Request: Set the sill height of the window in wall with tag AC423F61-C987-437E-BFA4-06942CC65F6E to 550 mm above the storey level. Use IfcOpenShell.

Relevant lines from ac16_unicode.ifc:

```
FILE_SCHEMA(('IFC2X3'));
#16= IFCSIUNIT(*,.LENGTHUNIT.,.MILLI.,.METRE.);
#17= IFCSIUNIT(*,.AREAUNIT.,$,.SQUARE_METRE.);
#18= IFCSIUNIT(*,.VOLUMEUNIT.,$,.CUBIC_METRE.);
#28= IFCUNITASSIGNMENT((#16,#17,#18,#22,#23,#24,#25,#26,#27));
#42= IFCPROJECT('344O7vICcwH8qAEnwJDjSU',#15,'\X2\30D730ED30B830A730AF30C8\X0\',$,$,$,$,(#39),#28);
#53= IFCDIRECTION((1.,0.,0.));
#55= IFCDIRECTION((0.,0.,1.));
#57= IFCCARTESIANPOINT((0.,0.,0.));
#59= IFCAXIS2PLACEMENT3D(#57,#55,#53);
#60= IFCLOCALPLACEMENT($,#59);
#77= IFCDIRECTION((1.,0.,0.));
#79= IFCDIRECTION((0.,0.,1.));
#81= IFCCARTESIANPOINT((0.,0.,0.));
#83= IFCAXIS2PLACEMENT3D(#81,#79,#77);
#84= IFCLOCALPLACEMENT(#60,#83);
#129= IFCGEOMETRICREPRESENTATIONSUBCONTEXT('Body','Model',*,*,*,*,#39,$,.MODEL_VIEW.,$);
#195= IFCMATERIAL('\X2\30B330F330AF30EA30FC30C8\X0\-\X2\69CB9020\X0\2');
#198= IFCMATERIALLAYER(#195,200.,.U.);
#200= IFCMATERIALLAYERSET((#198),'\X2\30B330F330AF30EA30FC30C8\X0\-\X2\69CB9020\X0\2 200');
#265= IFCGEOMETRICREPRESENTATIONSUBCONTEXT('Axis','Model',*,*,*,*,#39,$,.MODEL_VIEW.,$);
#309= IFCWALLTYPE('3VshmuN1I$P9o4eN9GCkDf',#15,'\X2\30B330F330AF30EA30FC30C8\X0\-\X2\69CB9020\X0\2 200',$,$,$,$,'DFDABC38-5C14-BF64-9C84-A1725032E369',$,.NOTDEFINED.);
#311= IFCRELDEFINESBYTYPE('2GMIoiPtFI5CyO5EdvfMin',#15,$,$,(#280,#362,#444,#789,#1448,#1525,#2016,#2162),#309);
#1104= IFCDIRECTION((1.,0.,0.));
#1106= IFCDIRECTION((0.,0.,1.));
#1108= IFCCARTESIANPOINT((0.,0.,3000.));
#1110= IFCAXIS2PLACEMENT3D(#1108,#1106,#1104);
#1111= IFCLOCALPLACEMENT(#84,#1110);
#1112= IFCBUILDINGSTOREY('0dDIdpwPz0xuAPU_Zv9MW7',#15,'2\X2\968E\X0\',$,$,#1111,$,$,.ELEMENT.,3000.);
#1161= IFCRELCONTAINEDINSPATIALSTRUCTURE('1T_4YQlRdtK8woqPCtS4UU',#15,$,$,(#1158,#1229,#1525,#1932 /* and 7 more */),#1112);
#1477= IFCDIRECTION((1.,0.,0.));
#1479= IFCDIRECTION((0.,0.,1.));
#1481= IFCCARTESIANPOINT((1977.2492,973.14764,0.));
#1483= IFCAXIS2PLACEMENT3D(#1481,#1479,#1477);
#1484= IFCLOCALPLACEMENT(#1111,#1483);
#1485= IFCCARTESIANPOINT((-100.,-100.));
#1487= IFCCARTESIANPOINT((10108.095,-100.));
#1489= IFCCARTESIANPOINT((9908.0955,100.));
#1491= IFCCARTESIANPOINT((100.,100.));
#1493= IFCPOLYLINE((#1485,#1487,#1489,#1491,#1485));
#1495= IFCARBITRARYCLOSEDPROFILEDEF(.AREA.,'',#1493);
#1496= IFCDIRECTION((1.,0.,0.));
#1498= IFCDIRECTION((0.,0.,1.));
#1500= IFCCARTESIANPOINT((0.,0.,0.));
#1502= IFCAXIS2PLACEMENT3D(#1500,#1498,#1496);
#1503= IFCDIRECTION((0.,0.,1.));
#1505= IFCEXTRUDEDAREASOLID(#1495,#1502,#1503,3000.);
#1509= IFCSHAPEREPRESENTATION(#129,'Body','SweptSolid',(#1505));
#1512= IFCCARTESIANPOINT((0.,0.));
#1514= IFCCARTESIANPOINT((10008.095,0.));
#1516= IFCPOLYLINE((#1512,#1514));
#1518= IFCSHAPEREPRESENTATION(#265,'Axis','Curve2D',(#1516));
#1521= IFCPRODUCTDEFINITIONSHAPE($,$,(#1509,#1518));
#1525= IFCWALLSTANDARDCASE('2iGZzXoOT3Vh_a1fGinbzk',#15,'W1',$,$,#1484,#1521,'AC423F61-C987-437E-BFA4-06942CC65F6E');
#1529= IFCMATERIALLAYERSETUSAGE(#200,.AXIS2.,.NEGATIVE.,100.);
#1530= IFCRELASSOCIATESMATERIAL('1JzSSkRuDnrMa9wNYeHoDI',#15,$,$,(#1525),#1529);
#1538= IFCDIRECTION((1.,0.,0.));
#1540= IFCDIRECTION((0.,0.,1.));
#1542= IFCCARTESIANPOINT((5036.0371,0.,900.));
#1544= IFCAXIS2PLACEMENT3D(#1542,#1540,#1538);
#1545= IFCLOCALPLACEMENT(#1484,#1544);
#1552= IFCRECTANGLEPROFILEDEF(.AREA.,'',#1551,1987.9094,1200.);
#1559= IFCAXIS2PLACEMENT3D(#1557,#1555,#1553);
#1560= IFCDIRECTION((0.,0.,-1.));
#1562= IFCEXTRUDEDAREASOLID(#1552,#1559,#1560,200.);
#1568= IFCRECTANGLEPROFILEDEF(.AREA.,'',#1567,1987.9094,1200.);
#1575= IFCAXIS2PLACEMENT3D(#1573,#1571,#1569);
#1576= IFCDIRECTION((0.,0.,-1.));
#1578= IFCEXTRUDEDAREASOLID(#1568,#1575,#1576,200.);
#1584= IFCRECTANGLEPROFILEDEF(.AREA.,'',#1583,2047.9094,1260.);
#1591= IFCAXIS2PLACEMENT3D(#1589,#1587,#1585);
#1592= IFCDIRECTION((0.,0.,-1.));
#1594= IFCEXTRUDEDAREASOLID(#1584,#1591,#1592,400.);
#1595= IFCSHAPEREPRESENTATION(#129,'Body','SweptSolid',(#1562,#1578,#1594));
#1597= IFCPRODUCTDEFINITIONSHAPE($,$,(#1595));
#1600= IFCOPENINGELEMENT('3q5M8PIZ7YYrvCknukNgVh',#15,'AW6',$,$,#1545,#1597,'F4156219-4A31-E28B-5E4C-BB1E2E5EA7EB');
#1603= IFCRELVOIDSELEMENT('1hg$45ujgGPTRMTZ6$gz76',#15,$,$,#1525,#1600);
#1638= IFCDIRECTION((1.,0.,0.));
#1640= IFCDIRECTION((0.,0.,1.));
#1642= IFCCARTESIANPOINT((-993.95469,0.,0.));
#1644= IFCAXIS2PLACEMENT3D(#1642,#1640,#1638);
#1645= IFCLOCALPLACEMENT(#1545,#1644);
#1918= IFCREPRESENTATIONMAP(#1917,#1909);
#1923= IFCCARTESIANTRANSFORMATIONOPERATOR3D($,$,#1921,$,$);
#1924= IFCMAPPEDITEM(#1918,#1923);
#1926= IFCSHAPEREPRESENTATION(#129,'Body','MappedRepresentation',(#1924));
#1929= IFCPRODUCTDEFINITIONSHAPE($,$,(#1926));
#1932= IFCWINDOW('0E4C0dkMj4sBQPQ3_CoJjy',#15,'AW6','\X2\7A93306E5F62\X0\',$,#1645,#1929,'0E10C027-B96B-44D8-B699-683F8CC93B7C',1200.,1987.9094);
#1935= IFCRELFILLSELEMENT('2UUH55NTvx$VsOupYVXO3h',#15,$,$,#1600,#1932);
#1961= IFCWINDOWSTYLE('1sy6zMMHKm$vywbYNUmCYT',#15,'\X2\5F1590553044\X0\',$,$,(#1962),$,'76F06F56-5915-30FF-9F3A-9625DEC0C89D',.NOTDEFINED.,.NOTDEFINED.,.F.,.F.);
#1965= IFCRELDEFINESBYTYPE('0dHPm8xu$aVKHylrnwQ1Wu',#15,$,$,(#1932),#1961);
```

```python
import numpy as np
import ifcopenshell
import ifcopenshell.api.geometry
import ifcopenshell.geom
import ifcopenshell.util.element
import ifcopenshell.util.placement
import ifcopenshell.util.shape
import ifcopenshell.util.unit

model = ifcopenshell.open("ac16_unicode.ifc")
unit_scale = ifcopenshell.util.unit.calculate_unit_scale(model)

window = model.by_id(1932)
opening = window.FillsVoids[0].RelatingOpeningElement
storey = ifcopenshell.util.element.get_container(window, ifc_class="IfcBuildingStorey")
level = ifcopenshell.util.placement.get_local_placement(storey.ObjectPlacement)[2, 3]

# The opening's origin need not be at the sill, so measure its lowest point.
shape = ifcopenshell.geom.create_shape(ifcopenshell.geom.settings(), opening)
bottom = ifcopenshell.util.shape.get_shape_bottom_elevation(shape, shape.geometry) / unit_scale
dz = level + 550.0 - bottom

shift = np.array([0.0, 0.0, dz])
# The window is placed relative to its opening, so it follows when the opening moves.
matrix = ifcopenshell.util.placement.get_local_placement(opening.ObjectPlacement)
matrix[:3, 3] += shift
ifcopenshell.api.geometry.edit_object_placement(
    model, product=opening, matrix=matrix, is_si=False, should_transform_children=True
)

print(f"moved by {dz * unit_scale:+.3f} m")

model.write("ac16_unicode_edited.ifc")
```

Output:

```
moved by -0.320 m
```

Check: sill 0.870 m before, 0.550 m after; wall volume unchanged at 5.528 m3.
